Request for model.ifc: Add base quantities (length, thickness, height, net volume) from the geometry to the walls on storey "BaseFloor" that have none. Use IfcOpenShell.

First a look at what the model holds.

```python
import ifcopenshell
import ifcopenshell.util.element
import ifcopenshell.util.unit

model = ifcopenshell.open("model.ifc")
print(model.schema)
for unit_type in ("LENGTHUNIT", "AREAUNIT", "VOLUMEUNIT"):
    print(unit_type, ifcopenshell.util.unit.calculate_unit_scale(model, unit_type))
storey = next(s for s in model.by_type("IfcBuildingStorey") if s.Name == "BaseFloor")
walls = [e for e in ifcopenshell.util.element.get_decomposition(storey) if e.is_a("IfcWall")]
for e in sorted(walls, key=lambda e: e.id()):
    print(e.id(), e.is_a(), e.Name, list(ifcopenshell.util.element.get_psets(e, qtos_only=True)), sep=" | ")
```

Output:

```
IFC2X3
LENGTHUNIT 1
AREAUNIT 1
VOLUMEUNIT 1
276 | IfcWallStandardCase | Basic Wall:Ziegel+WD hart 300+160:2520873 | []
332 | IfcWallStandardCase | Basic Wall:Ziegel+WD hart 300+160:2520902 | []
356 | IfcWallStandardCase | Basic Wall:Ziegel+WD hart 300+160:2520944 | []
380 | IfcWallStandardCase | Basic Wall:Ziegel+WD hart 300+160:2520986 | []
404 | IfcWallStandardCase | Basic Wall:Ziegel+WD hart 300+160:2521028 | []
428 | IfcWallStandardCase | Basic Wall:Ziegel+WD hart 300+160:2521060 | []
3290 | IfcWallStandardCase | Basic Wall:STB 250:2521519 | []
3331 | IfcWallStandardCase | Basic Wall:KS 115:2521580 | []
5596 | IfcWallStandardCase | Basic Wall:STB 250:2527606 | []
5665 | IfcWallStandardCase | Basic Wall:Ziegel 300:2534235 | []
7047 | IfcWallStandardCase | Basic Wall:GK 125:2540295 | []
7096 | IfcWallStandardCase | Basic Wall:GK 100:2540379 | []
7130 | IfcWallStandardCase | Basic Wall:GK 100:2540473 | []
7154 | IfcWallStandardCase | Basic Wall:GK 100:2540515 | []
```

```python
import ifcopenshell
import ifcopenshell.api.pset
import ifcopenshell.geom
import ifcopenshell.util.element
import ifcopenshell.util.shape
import ifcopenshell.util.unit

model = ifcopenshell.open("model.ifc")
unit_scale = ifcopenshell.util.unit.calculate_unit_scale(model)
volume_scale = ifcopenshell.util.unit.calculate_unit_scale(model, "VOLUMEUNIT")
settings = ifcopenshell.geom.settings()

storey = next(s for s in model.by_type("IfcBuildingStorey") if s.Name == "BaseFloor")
walls = [e for e in ifcopenshell.util.element.get_decomposition(storey) if e.is_a("IfcWall")]

for e in sorted(walls, key=lambda e: e.id()):
    if ifcopenshell.util.element.get_psets(e, qtos_only=True, should_inherit=False):
        continue
    # Geometry comes back in metres, in the element's own axes.
    shape = ifcopenshell.geom.create_shape(settings, e)
    values = {
        "Length": ifcopenshell.util.shape.get_x(shape.geometry) / unit_scale,
        "Width": ifcopenshell.util.shape.get_y(shape.geometry) / unit_scale,
        "Height": ifcopenshell.util.shape.get_z(shape.geometry) / unit_scale,
        "NetVolume": ifcopenshell.util.shape.get_volume(shape.geometry) / volume_scale,
    }
    qto = ifcopenshell.api.pset.add_qto(model, product=e, name="BaseQuantities")
    ifcopenshell.api.pset.edit_qto(model, qto=qto, properties=values)
    print(e.id(), {k: round(v, 3) for k, v in values.items()})

model.write("model_edited.ifc")
```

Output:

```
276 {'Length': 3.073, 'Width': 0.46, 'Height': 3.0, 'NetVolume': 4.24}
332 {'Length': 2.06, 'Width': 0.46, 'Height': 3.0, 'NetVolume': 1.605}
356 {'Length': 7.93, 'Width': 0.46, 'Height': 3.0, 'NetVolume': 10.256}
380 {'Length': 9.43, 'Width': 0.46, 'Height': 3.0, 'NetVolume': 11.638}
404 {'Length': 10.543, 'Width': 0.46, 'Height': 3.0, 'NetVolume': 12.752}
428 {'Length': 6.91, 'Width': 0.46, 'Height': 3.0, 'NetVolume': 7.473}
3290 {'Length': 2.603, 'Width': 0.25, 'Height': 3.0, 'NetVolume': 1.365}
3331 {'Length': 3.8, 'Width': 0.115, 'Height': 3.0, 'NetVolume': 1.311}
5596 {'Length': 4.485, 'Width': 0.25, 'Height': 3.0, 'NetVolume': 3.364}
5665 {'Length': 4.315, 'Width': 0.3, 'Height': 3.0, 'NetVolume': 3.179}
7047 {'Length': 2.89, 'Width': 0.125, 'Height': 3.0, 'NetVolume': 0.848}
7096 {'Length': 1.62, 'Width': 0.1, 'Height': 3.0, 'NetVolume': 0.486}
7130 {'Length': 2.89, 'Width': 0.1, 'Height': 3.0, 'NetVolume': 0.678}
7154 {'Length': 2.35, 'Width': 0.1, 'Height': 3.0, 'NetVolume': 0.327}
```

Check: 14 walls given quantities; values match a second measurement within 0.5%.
